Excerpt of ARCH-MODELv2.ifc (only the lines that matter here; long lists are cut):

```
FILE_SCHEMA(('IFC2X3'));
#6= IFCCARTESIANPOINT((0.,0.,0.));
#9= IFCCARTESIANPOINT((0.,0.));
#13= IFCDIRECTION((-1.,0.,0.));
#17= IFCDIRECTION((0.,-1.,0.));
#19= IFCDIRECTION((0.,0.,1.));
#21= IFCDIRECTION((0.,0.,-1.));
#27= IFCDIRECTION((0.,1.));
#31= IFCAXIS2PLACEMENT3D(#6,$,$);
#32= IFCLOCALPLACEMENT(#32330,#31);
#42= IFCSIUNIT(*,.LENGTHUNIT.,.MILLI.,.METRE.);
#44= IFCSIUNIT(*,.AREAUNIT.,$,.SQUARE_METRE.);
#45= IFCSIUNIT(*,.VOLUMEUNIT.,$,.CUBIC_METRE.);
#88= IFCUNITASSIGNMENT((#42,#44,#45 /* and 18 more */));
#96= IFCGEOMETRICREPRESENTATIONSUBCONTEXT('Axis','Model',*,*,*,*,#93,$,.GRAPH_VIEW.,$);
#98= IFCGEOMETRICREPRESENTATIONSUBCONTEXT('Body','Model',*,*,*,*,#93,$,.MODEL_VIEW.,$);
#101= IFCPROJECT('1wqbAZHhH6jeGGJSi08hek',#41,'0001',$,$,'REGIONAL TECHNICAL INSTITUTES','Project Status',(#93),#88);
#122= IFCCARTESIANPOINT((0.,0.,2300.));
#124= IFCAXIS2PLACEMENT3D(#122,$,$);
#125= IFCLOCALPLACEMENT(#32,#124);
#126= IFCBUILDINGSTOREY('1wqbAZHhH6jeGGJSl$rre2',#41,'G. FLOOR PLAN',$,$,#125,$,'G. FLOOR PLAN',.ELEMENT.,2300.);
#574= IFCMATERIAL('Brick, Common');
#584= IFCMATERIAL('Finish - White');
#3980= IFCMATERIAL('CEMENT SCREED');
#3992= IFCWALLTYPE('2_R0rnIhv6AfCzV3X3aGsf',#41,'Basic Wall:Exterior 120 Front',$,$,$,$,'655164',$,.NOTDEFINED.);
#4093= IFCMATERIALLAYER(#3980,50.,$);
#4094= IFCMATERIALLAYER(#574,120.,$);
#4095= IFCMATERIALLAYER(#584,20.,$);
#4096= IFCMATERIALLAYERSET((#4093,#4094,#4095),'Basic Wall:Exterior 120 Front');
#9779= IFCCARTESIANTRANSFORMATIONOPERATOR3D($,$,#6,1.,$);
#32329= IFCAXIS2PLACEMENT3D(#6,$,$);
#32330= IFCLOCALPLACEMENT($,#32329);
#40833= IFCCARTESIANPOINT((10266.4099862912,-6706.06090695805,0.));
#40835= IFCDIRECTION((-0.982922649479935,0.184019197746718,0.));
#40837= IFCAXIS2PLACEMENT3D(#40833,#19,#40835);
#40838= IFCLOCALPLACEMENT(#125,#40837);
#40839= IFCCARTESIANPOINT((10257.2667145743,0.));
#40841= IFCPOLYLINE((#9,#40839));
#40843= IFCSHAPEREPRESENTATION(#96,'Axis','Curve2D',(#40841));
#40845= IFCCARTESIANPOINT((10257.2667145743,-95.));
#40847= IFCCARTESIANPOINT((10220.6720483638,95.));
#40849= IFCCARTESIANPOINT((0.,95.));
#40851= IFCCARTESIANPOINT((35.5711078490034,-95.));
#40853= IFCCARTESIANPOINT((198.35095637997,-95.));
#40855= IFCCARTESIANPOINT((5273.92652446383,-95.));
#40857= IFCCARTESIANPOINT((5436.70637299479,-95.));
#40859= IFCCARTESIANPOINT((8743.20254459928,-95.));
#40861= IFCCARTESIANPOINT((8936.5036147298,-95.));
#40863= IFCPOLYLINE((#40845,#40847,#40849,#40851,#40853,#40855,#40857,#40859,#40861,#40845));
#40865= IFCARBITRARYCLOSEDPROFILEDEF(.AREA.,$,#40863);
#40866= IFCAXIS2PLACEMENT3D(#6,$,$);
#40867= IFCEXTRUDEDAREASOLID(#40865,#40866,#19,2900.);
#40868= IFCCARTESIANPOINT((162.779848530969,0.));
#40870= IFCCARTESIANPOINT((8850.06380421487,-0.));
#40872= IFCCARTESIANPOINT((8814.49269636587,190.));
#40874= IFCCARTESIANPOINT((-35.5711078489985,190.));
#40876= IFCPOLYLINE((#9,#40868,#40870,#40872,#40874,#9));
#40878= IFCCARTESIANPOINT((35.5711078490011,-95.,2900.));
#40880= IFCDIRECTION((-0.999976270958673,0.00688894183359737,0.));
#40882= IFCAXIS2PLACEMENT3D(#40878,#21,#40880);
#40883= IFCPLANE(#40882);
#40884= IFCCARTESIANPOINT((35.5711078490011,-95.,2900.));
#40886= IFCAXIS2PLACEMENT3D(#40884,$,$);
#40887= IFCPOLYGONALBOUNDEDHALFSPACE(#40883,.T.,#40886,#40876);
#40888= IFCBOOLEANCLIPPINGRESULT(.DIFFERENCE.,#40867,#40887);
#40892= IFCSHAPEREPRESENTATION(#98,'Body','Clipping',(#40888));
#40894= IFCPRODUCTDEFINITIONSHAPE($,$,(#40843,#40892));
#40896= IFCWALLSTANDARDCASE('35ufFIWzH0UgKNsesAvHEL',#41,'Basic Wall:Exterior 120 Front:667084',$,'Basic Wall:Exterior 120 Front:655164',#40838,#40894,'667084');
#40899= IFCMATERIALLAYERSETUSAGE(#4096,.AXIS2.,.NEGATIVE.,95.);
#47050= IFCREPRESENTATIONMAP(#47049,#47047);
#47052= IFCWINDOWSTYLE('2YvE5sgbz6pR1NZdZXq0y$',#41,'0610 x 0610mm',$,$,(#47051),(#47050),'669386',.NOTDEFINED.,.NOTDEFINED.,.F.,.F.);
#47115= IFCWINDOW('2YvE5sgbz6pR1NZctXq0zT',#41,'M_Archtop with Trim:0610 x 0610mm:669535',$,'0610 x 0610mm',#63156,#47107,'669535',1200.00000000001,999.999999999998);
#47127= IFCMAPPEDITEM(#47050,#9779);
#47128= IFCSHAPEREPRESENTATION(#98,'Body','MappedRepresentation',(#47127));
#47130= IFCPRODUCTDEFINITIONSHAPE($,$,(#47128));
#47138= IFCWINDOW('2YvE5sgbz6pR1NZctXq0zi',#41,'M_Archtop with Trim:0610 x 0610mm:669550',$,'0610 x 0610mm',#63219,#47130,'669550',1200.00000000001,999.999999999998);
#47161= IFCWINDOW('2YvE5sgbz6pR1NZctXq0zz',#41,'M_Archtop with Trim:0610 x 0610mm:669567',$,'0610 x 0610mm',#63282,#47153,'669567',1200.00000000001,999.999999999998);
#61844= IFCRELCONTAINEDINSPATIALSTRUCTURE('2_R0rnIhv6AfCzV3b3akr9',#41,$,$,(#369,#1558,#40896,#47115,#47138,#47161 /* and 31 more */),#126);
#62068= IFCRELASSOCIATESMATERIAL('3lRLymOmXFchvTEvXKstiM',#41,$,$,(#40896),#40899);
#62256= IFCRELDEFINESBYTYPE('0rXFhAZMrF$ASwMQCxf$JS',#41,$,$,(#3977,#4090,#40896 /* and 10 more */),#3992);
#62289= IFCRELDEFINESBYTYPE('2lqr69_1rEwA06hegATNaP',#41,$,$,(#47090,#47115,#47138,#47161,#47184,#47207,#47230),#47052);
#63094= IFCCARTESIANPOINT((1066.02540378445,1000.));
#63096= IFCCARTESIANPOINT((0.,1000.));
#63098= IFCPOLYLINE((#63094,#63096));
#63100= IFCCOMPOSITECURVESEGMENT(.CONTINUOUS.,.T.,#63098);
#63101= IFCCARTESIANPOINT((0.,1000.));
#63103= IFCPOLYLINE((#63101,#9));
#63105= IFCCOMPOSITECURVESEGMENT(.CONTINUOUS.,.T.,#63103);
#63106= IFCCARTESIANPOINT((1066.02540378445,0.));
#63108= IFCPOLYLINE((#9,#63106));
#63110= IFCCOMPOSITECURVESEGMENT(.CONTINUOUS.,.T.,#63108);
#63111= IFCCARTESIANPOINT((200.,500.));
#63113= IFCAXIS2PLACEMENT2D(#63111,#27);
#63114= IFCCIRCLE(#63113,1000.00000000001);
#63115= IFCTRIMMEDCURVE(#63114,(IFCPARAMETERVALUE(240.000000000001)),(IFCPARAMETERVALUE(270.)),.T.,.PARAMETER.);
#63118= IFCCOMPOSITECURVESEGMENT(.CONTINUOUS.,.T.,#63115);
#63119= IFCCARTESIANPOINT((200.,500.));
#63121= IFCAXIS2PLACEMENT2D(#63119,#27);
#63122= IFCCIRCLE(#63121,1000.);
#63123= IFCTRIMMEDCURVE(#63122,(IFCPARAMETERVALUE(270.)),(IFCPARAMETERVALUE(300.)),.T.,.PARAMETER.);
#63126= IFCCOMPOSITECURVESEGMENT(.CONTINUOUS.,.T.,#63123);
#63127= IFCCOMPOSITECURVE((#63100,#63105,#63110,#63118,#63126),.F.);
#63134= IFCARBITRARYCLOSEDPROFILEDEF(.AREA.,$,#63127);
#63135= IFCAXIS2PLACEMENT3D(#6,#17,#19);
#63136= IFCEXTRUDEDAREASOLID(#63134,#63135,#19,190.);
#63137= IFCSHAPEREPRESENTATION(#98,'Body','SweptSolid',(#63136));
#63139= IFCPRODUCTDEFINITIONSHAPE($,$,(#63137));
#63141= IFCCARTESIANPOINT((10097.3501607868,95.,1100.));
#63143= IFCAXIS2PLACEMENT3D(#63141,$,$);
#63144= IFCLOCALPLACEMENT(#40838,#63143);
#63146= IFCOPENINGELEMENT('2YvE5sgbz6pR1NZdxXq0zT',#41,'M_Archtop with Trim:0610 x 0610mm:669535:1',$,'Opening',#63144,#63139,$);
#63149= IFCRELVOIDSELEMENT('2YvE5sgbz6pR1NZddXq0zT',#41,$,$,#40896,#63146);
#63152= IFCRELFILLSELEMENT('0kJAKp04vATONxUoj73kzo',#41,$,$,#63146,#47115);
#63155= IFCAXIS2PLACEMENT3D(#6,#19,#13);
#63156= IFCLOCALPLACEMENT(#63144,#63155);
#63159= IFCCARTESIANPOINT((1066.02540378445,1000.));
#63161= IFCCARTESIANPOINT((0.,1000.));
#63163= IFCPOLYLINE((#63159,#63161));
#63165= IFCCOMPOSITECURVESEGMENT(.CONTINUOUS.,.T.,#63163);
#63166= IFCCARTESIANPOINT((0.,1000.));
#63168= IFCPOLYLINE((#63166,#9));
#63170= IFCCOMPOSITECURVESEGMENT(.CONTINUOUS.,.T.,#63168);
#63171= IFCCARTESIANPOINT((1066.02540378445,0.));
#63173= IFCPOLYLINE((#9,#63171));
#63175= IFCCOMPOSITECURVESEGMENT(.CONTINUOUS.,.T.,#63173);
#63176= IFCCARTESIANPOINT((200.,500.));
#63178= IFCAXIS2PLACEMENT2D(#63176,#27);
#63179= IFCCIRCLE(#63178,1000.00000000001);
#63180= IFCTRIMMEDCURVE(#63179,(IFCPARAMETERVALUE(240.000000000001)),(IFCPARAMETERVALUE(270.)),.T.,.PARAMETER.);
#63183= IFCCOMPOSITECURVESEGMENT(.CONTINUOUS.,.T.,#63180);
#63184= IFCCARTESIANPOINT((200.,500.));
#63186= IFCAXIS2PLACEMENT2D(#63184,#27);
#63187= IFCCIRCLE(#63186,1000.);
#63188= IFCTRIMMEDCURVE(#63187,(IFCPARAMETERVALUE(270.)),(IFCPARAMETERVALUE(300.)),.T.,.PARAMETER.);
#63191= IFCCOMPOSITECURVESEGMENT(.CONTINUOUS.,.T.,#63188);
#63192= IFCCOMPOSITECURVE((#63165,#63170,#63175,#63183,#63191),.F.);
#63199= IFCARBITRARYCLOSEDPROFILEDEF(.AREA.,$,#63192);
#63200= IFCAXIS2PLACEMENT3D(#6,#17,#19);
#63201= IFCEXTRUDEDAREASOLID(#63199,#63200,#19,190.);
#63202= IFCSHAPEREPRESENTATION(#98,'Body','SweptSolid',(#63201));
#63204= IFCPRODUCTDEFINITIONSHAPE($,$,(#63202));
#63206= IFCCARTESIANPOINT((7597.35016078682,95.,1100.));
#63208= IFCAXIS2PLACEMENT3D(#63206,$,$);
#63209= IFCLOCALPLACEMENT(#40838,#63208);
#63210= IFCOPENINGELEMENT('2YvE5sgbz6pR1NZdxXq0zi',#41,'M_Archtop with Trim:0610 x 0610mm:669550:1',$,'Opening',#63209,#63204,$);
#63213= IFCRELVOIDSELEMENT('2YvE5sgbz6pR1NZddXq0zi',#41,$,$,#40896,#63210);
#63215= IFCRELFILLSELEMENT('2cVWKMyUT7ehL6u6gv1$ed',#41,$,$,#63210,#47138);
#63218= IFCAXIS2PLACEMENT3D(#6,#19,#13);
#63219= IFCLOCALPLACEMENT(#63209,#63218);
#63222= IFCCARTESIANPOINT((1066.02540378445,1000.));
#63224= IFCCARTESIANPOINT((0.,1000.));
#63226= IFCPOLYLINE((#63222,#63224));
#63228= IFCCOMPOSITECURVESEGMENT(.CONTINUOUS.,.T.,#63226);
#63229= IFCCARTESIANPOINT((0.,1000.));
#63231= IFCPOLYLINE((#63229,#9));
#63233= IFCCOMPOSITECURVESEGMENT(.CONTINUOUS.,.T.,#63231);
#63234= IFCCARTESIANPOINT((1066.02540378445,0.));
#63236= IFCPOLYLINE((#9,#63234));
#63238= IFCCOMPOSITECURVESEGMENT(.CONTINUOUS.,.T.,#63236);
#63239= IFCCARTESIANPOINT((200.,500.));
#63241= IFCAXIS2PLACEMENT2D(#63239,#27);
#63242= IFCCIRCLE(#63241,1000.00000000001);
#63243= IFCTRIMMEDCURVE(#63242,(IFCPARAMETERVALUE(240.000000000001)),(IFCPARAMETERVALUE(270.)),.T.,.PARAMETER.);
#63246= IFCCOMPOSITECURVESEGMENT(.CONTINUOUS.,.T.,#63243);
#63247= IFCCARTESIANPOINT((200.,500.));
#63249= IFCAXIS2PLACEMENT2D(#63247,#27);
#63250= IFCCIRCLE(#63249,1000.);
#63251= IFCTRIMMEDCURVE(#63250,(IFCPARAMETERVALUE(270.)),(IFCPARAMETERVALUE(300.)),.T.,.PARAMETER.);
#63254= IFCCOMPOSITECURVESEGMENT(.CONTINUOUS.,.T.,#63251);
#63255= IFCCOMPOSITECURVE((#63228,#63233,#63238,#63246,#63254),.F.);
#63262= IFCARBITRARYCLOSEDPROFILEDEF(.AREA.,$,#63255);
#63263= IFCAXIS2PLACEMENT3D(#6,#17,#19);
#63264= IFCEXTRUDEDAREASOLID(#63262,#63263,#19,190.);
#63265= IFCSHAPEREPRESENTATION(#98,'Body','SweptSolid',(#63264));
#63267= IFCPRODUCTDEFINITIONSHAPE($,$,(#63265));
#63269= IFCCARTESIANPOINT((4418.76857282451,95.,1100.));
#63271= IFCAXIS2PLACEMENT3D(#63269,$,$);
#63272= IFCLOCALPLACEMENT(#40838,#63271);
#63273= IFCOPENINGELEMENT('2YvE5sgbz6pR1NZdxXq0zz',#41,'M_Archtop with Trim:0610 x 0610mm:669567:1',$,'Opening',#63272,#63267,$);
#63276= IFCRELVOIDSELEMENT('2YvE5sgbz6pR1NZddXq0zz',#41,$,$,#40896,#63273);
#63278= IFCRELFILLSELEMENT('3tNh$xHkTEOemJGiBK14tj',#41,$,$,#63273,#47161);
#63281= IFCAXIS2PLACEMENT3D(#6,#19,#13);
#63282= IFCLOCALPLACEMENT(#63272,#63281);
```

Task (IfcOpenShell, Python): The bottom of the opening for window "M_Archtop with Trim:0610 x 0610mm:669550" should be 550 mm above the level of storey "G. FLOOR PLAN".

```python
import numpy as np
import ifcopenshell
import ifcopenshell.api.geometry
import ifcopenshell.geom
import ifcopenshell.util.element
import ifcopenshell.util.placement
import ifcopenshell.util.shape
import ifcopenshell.util.unit

model = ifcopenshell.open("ARCH-MODELv2.ifc")
unit_scale = ifcopenshell.util.unit.calculate_unit_scale(model)

window = model.by_id(47138)
opening = window.FillsVoids[0].RelatingOpeningElement
storey = ifcopenshell.util.element.get_container(window, ifc_class="IfcBuildingStorey")
level = ifcopenshell.util.placement.get_local_placement(storey.ObjectPlacement)[2, 3]

# The opening's origin need not be at the sill, so measure its lowest point.
shape = ifcopenshell.geom.create_shape(ifcopenshell.geom.settings(), opening)
bottom = ifcopenshell.util.shape.get_shape_bottom_elevation(shape, shape.geometry) / unit_scale
dz = level + 0.55 / unit_scale - bottom

shift = np.array([0.0, 0.0, dz])
# The window is placed relative to its opening, so it follows when the opening moves.
matrix = ifcopenshell.util.placement.get_local_placement(opening.ObjectPlacement)
matrix[:3, 3] += shift
ifcopenshell.api.geometry.edit_object_placement(
    model, product=opening, matrix=matrix, is_si=False, should_transform_children=True
)

print(f"moved by {dz * unit_scale:+.3f} m")

model.write("ARCH-MODELv2_v2.ifc")
```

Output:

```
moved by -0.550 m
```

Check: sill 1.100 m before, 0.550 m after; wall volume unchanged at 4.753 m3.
